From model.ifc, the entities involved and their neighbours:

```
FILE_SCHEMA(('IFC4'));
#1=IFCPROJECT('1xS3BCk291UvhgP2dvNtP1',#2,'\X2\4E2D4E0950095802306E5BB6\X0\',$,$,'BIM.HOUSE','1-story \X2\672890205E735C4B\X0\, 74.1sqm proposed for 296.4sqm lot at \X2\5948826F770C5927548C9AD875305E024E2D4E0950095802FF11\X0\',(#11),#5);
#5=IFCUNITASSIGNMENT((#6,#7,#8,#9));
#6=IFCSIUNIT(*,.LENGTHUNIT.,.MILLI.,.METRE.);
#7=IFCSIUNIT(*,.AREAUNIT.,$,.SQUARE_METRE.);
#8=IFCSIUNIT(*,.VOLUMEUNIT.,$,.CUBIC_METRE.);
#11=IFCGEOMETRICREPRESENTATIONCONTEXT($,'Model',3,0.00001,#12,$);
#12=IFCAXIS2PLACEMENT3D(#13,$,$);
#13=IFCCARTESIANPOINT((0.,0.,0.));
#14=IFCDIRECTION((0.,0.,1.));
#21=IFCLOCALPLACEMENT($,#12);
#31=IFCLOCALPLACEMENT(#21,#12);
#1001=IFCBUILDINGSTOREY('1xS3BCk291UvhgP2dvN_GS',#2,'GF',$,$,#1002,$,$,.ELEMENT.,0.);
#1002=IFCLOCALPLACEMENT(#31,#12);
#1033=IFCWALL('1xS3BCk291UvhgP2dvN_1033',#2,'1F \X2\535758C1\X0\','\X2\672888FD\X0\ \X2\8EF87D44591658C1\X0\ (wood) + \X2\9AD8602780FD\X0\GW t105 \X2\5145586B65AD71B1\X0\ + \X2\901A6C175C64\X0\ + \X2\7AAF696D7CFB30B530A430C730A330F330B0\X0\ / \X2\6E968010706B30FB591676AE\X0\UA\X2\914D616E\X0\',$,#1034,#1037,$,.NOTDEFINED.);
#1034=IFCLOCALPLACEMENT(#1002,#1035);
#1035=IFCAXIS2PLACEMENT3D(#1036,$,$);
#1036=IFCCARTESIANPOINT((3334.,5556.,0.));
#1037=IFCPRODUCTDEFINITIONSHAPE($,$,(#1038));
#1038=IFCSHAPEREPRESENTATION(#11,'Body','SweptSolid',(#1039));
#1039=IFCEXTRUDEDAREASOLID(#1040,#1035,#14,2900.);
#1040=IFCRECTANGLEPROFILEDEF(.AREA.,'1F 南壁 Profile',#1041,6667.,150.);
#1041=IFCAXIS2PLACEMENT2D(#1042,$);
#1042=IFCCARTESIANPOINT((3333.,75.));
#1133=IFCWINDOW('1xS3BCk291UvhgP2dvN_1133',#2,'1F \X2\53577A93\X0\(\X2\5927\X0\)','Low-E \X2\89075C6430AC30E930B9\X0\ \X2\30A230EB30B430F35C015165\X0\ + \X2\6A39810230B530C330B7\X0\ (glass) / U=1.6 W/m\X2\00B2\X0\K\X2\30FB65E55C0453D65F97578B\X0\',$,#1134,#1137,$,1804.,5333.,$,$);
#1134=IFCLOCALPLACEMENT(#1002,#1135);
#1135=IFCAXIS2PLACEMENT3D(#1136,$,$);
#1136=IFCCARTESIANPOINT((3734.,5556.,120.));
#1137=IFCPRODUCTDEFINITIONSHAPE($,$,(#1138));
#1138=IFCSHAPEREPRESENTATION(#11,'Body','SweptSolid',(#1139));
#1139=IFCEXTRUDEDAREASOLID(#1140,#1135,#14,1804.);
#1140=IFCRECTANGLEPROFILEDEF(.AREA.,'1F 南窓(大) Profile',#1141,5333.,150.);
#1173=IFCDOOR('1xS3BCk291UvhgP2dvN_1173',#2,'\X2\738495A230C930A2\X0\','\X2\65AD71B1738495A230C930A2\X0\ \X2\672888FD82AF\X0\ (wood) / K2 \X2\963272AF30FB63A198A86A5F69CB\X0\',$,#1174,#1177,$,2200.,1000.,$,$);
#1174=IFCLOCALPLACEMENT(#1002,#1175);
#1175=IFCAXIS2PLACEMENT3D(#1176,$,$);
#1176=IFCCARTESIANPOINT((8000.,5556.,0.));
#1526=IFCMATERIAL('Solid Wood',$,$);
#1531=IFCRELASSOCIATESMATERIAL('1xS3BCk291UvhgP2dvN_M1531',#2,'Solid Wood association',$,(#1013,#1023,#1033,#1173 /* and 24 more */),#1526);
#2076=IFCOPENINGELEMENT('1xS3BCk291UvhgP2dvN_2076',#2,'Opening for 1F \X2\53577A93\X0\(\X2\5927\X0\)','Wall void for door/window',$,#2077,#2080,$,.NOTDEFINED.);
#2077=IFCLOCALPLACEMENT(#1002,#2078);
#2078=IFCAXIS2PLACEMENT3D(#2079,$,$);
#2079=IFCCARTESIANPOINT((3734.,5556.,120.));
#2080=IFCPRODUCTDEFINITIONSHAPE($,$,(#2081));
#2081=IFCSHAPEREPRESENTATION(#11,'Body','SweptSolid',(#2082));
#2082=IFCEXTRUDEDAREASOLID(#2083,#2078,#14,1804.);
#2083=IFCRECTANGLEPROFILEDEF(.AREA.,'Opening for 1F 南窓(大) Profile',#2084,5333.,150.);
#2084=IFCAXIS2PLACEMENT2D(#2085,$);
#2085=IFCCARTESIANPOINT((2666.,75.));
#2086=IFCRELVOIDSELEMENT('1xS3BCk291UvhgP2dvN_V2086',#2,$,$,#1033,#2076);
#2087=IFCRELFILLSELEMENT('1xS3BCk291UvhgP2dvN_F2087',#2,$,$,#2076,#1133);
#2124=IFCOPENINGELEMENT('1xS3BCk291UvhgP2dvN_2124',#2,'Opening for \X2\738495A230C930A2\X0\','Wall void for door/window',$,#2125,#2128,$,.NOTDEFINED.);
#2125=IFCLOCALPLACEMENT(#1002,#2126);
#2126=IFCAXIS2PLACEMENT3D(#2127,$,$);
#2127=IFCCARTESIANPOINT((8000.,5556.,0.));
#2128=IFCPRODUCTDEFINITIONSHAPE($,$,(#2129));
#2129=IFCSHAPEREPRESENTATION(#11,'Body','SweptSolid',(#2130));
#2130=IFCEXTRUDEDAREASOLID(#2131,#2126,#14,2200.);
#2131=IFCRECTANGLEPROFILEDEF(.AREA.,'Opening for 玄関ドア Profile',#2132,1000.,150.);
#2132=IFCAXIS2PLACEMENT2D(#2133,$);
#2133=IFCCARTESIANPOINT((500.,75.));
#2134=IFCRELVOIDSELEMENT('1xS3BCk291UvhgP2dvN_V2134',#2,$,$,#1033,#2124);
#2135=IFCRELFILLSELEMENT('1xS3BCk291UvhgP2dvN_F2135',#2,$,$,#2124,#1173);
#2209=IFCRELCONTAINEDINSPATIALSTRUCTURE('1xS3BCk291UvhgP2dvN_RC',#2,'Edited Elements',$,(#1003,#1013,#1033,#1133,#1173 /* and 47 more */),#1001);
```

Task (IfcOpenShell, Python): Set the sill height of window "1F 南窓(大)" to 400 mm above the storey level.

```python
import numpy as np
import ifcopenshell
import ifcopenshell.api.geometry
import ifcopenshell.geom
import ifcopenshell.util.element
import ifcopenshell.util.placement
import ifcopenshell.util.shape
import ifcopenshell.util.unit

model = ifcopenshell.open("model.ifc")
unit_scale = ifcopenshell.util.unit.calculate_unit_scale(model)

window = model.by_guid("1xS3BCk291UvhgP2dvN_1133")
opening = window.FillsVoids[0].RelatingOpeningElement
storey = ifcopenshell.util.element.get_container(window, ifc_class="IfcBuildingStorey")
level = ifcopenshell.util.placement.get_local_placement(storey.ObjectPlacement)[2, 3]

# The opening's origin need not be at the sill, so measure its lowest point.
shape = ifcopenshell.geom.create_shape(ifcopenshell.geom.settings(), opening)
bottom = ifcopenshell.util.shape.get_shape_bottom_elevation(shape, shape.geometry) / unit_scale
dz = level + 400.0 - bottom

shift = np.array([0.0, 0.0, dz])
# The window is not placed relative to its opening, so move both.
for product in (opening, window):
    matrix = ifcopenshell.util.placement.get_local_placement(product.ObjectPlacement)
    matrix[:3, 3] += shift
    ifcopenshell.api.geometry.edit_object_placement(model, product=product, matrix=matrix, is_si=False)

print(f"moved by {dz * unit_scale:+.3f} m")

model.write("model-out.ifc")
```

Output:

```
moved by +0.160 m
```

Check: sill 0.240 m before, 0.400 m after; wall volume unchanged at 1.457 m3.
